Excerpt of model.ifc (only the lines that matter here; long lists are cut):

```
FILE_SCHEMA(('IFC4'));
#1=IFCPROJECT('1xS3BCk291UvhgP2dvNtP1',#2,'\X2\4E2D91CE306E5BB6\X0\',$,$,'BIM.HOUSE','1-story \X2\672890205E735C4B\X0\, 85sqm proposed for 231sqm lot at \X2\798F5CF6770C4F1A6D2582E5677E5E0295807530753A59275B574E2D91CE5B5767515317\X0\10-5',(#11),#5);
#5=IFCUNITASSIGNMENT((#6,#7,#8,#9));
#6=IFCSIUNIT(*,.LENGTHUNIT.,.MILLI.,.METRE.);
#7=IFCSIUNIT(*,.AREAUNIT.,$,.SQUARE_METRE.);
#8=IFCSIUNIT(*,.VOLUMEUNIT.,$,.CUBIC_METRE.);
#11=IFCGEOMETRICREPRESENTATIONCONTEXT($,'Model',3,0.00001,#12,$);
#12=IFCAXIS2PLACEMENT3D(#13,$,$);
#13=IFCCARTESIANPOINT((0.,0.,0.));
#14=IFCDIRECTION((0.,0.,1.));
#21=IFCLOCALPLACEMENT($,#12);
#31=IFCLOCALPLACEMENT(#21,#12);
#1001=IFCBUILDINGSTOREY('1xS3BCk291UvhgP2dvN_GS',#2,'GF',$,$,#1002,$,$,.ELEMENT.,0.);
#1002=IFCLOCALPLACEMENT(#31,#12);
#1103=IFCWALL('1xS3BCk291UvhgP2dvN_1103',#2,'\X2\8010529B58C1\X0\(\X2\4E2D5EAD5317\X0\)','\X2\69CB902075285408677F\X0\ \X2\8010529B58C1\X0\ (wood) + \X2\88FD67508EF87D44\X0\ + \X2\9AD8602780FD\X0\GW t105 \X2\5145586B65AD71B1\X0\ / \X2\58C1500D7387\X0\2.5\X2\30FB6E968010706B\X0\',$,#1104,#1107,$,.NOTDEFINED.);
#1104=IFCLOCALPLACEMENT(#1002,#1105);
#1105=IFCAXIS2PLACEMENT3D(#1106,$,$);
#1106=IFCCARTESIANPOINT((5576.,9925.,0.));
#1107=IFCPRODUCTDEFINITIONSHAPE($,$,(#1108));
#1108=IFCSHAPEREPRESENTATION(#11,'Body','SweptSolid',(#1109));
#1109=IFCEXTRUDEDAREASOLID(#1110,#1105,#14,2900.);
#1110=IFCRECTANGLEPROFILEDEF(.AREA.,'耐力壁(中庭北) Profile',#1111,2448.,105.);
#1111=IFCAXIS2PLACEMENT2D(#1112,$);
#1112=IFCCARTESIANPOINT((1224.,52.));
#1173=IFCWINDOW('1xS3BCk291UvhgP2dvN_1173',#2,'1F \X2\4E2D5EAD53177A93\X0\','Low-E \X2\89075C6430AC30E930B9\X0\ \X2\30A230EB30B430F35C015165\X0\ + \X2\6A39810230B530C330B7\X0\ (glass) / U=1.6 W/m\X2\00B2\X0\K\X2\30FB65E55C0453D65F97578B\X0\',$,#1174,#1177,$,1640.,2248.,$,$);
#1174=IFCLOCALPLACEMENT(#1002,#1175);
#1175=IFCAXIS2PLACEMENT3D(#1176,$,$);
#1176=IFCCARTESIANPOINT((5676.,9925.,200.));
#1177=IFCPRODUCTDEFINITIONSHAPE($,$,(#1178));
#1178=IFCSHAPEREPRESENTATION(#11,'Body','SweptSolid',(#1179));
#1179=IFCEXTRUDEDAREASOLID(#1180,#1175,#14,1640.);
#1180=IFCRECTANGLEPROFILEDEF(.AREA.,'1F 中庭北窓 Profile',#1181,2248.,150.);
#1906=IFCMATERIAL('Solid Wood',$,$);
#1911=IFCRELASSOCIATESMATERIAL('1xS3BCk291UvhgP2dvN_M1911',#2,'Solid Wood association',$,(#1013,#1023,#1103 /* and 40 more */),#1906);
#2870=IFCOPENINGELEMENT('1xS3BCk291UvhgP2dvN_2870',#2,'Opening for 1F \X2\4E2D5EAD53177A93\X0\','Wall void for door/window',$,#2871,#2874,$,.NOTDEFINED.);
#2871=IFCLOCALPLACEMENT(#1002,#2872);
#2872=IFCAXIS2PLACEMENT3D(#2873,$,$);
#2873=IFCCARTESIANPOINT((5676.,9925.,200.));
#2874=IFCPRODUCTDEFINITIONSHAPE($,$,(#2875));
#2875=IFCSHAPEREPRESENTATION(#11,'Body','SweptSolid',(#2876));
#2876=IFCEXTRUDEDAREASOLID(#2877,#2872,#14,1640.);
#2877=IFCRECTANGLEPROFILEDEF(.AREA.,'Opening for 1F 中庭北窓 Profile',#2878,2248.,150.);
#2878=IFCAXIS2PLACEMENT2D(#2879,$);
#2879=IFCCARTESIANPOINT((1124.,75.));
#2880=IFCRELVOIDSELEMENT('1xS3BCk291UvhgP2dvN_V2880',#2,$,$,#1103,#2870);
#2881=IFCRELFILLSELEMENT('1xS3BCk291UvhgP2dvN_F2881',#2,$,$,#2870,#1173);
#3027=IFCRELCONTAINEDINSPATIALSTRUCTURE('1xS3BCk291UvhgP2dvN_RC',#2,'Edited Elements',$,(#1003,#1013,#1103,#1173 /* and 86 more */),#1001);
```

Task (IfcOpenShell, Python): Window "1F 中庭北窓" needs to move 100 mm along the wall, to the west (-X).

```python
import ifcopenshell
import ifcopenshell.api.geometry
import ifcopenshell.util.placement
import ifcopenshell.util.unit

model = ifcopenshell.open("model.ifc")
unit_scale = ifcopenshell.util.unit.calculate_unit_scale(model)

window = model.by_guid("1xS3BCk291UvhgP2dvN_1173")
opening = window.FillsVoids[0].RelatingOpeningElement
wall = opening.VoidsElements[0].RelatingBuildingElement

wall_matrix = ifcopenshell.util.placement.get_local_placement(wall.ObjectPlacement)
shift = wall_matrix[:3, 0] * -0.1 / unit_scale
before = ifcopenshell.util.placement.get_local_placement(window.ObjectPlacement)[:3, 3].copy()

# The window is not placed relative to its opening, so move both.
for product in (opening, window):
    matrix = ifcopenshell.util.placement.get_local_placement(product.ObjectPlacement)
    matrix[:3, 3] += shift
    ifcopenshell.api.geometry.edit_object_placement(model, product=product, matrix=matrix, is_si=False)

after = ifcopenshell.util.placement.get_local_placement(window.ObjectPlacement)[:3, 3]
print("window moved by", (after - before).round(3) + 0.0)

model.write("model_rev.ifc")
```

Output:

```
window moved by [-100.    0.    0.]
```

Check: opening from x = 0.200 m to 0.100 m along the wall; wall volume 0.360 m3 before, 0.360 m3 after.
